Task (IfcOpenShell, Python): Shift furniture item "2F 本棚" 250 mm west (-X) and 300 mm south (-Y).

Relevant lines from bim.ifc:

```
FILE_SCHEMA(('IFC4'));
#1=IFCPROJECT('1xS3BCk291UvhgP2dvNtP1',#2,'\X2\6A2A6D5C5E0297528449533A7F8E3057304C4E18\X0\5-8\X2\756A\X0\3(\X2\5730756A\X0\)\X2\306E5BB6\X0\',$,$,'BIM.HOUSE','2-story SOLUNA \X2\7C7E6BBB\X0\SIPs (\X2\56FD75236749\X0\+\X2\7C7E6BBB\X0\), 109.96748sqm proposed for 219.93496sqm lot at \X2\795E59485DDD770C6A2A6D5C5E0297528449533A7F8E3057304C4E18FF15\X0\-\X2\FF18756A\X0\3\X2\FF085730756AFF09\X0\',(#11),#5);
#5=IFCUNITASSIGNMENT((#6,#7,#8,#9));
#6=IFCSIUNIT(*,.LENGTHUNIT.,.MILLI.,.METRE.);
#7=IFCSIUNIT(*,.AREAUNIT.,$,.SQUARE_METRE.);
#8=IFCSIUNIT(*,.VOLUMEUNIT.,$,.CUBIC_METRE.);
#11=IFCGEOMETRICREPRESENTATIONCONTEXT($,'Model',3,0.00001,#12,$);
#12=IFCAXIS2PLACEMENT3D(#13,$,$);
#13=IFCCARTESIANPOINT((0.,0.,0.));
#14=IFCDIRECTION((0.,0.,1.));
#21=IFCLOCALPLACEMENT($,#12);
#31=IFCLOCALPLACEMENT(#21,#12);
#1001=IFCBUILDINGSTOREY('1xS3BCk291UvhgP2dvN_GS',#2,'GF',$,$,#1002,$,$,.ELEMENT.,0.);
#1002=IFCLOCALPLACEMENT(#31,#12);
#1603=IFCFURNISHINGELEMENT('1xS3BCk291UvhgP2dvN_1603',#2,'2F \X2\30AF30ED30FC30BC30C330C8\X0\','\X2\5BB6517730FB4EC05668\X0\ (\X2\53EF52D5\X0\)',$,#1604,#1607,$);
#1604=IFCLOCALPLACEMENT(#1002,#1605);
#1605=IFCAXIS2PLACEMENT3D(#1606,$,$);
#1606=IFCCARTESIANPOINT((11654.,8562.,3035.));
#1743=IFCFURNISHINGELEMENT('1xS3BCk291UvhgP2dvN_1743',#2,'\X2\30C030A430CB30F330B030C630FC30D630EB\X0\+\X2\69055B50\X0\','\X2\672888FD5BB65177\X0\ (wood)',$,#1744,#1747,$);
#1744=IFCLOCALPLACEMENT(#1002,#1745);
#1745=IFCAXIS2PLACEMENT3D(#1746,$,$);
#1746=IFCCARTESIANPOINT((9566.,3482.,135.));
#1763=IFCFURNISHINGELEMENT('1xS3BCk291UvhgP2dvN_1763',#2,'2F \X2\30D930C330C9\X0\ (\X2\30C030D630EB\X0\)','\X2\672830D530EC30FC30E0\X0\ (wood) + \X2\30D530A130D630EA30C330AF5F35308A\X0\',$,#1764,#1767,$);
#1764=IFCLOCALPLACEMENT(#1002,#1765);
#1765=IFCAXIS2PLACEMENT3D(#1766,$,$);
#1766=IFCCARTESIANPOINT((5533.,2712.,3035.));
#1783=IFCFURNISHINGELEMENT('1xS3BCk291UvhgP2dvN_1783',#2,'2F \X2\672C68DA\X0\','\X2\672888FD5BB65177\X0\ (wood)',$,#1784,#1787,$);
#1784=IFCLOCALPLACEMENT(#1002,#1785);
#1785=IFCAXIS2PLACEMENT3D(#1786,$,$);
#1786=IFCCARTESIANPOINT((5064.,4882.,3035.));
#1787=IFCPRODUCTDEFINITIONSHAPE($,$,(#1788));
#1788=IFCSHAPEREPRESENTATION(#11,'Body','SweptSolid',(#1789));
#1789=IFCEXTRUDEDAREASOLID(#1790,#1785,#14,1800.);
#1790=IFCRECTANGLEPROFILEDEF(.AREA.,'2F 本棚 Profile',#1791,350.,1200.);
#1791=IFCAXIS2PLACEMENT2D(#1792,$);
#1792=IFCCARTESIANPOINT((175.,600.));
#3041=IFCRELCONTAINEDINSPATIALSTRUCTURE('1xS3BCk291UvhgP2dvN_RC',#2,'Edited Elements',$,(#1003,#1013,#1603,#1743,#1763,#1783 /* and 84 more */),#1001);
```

```python
import ifcopenshell
import ifcopenshell.api.geometry
import ifcopenshell.util.placement

model = ifcopenshell.open("bim.ifc")

item = model.by_guid("1xS3BCk291UvhgP2dvN_1783")
matrix = ifcopenshell.util.placement.get_local_placement(item.ObjectPlacement)
matrix[0, 3] -= 250.0
matrix[1, 3] -= 300.0
ifcopenshell.api.geometry.edit_object_placement(model, product=item, matrix=matrix, is_si=False)

print(ifcopenshell.util.placement.get_local_placement(item.ObjectPlacement).round(3) + 0.0)

model.write("bim-out.ifc")
```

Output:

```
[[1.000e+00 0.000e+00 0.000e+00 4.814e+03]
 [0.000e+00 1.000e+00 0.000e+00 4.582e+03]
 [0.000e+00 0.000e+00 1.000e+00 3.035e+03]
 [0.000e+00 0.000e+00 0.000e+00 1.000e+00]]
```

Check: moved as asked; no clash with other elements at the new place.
